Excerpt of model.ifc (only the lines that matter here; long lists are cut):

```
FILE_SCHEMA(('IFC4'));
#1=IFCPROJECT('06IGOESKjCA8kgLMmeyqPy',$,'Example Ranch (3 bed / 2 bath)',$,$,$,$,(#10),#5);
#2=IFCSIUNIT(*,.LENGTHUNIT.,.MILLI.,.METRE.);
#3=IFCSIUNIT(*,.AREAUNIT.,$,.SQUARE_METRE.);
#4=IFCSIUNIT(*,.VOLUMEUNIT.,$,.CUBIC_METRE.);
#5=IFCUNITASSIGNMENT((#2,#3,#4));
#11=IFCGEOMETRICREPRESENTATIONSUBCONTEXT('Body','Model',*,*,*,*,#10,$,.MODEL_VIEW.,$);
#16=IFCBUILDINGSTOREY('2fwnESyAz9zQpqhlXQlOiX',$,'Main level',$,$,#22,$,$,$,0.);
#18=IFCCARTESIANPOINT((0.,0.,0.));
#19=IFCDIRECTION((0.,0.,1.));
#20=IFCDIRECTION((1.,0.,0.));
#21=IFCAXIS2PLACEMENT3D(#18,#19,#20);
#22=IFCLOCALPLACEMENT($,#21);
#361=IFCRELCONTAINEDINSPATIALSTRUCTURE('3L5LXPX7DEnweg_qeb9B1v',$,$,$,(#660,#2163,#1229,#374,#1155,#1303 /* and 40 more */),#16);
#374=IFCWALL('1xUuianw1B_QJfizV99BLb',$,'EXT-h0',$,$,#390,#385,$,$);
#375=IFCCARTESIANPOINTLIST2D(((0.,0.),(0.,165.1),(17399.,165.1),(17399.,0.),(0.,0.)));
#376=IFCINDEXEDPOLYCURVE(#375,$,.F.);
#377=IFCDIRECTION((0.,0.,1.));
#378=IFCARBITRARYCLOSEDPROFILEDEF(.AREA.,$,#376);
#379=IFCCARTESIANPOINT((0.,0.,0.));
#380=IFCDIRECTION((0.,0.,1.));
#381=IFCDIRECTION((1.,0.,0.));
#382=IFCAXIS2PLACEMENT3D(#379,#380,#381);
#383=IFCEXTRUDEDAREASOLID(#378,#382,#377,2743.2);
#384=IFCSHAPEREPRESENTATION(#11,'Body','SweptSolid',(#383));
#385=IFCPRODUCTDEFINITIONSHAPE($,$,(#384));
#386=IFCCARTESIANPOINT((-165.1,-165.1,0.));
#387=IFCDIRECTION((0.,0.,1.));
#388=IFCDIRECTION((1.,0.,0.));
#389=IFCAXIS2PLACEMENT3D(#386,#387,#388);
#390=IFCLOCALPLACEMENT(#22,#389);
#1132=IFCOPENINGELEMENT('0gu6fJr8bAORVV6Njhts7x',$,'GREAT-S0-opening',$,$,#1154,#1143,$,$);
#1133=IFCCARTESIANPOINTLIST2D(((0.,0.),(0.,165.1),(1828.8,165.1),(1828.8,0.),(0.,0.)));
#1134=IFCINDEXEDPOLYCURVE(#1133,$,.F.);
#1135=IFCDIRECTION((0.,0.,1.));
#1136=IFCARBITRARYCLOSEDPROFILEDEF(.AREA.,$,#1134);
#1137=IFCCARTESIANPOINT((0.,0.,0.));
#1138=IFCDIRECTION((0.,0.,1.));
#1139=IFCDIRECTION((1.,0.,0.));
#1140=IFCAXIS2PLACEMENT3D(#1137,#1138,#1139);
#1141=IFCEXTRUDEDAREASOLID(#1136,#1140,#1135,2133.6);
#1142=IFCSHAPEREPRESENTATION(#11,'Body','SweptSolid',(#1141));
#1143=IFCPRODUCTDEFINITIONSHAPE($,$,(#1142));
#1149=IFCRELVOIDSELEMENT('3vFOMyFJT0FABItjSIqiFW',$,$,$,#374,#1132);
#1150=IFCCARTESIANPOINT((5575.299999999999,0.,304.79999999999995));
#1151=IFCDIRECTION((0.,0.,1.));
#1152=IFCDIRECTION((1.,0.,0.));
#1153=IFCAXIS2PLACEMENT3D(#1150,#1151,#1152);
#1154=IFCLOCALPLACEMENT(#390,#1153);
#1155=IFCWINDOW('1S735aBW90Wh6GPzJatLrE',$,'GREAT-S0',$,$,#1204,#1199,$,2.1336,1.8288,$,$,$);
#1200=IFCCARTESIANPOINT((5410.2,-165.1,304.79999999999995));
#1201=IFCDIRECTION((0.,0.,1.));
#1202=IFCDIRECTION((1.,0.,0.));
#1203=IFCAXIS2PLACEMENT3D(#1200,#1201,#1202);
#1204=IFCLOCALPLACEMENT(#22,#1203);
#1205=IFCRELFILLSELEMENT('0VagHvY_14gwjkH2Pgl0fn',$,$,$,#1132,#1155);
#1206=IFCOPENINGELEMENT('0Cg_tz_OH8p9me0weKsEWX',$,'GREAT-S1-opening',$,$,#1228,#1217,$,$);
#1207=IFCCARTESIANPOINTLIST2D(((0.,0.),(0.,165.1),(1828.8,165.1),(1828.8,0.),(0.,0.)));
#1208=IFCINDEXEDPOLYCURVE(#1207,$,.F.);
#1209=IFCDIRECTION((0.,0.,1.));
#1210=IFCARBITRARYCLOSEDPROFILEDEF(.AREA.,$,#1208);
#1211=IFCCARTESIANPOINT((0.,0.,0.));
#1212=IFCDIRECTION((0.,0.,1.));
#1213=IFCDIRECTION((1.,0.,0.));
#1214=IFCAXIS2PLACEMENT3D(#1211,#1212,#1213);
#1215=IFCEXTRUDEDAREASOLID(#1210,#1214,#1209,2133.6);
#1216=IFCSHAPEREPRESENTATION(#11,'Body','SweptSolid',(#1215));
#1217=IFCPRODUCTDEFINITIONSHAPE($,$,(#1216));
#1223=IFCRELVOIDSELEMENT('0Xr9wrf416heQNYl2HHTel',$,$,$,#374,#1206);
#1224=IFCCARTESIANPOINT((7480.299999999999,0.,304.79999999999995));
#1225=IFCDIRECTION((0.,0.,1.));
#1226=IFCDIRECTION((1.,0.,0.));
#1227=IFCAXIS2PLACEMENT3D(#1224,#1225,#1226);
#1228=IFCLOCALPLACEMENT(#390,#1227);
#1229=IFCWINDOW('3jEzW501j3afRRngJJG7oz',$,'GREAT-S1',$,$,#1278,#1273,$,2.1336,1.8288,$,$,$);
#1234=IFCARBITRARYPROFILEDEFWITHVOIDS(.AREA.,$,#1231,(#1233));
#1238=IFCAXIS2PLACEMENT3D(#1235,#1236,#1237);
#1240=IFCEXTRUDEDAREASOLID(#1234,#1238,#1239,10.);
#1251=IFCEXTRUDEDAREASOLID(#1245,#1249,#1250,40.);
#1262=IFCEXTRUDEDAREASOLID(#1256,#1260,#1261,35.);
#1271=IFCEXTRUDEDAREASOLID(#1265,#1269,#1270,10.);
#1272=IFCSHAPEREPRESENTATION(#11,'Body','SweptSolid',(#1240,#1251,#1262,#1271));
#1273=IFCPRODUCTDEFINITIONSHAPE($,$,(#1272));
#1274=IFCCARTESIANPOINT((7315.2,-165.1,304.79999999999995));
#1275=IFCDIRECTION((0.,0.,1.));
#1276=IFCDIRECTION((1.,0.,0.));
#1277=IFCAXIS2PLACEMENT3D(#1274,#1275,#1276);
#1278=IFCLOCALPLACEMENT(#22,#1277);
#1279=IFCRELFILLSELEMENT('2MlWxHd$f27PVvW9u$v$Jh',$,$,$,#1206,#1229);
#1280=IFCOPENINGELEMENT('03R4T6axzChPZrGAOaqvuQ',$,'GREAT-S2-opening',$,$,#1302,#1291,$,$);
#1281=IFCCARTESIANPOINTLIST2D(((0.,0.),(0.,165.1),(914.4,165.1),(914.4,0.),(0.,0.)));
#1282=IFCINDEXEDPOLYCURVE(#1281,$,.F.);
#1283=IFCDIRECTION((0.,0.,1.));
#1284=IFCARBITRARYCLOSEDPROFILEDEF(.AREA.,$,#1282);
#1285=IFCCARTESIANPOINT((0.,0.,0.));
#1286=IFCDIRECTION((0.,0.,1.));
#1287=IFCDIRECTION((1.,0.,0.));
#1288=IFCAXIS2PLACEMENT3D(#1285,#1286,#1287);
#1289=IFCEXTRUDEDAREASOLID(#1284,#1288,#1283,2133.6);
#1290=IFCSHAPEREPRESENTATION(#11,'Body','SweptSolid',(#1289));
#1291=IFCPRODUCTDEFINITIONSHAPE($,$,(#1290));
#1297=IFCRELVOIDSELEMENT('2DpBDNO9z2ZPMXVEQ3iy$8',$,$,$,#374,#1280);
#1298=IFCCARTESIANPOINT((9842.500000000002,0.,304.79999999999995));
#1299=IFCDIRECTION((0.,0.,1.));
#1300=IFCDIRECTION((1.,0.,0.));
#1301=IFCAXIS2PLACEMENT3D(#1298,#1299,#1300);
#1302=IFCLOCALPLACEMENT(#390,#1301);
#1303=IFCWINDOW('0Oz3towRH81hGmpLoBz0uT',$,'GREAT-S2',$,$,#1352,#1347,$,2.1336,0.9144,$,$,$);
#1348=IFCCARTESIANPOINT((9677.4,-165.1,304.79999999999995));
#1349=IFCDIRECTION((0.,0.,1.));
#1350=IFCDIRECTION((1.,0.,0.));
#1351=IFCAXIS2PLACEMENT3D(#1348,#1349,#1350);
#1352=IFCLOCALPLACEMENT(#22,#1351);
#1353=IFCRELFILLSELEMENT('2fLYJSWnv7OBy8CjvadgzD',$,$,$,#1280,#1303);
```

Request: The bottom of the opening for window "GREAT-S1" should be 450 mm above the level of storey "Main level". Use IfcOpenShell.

```python
import numpy as np
import ifcopenshell
import ifcopenshell.api.geometry
import ifcopenshell.geom
import ifcopenshell.util.element
import ifcopenshell.util.placement
import ifcopenshell.util.shape
import ifcopenshell.util.unit

model = ifcopenshell.open("model.ifc")
unit_scale = ifcopenshell.util.unit.calculate_unit_scale(model)

window = model.by_guid("3jEzW501j3afRRngJJG7oz")
opening = window.FillsVoids[0].RelatingOpeningElement
storey = ifcopenshell.util.element.get_container(window, ifc_class="IfcBuildingStorey")
level = ifcopenshell.util.placement.get_local_placement(storey.ObjectPlacement)[2, 3]

# The opening's origin need not be at the sill, so measure its lowest point.
shape = ifcopenshell.geom.create_shape(ifcopenshell.geom.settings(), opening)
bottom = ifcopenshell.util.shape.get_shape_bottom_elevation(shape, shape.geometry) / unit_scale
dz = level + 0.45 / unit_scale - bottom

shift = np.array([0.0, 0.0, dz])
# The window is not placed relative to its opening, so move both.
for product in (opening, window):
    matrix = ifcopenshell.util.placement.get_local_placement(product.ObjectPlacement)
    matrix[:3, 3] += shift
    ifcopenshell.api.geometry.edit_object_placement(model, product=product, matrix=matrix, is_si=False)

print(f"moved by {dz * unit_scale:+.3f} m")

model.write("model_v2.ifc")
```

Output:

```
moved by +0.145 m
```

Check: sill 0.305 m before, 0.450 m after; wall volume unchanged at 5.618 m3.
